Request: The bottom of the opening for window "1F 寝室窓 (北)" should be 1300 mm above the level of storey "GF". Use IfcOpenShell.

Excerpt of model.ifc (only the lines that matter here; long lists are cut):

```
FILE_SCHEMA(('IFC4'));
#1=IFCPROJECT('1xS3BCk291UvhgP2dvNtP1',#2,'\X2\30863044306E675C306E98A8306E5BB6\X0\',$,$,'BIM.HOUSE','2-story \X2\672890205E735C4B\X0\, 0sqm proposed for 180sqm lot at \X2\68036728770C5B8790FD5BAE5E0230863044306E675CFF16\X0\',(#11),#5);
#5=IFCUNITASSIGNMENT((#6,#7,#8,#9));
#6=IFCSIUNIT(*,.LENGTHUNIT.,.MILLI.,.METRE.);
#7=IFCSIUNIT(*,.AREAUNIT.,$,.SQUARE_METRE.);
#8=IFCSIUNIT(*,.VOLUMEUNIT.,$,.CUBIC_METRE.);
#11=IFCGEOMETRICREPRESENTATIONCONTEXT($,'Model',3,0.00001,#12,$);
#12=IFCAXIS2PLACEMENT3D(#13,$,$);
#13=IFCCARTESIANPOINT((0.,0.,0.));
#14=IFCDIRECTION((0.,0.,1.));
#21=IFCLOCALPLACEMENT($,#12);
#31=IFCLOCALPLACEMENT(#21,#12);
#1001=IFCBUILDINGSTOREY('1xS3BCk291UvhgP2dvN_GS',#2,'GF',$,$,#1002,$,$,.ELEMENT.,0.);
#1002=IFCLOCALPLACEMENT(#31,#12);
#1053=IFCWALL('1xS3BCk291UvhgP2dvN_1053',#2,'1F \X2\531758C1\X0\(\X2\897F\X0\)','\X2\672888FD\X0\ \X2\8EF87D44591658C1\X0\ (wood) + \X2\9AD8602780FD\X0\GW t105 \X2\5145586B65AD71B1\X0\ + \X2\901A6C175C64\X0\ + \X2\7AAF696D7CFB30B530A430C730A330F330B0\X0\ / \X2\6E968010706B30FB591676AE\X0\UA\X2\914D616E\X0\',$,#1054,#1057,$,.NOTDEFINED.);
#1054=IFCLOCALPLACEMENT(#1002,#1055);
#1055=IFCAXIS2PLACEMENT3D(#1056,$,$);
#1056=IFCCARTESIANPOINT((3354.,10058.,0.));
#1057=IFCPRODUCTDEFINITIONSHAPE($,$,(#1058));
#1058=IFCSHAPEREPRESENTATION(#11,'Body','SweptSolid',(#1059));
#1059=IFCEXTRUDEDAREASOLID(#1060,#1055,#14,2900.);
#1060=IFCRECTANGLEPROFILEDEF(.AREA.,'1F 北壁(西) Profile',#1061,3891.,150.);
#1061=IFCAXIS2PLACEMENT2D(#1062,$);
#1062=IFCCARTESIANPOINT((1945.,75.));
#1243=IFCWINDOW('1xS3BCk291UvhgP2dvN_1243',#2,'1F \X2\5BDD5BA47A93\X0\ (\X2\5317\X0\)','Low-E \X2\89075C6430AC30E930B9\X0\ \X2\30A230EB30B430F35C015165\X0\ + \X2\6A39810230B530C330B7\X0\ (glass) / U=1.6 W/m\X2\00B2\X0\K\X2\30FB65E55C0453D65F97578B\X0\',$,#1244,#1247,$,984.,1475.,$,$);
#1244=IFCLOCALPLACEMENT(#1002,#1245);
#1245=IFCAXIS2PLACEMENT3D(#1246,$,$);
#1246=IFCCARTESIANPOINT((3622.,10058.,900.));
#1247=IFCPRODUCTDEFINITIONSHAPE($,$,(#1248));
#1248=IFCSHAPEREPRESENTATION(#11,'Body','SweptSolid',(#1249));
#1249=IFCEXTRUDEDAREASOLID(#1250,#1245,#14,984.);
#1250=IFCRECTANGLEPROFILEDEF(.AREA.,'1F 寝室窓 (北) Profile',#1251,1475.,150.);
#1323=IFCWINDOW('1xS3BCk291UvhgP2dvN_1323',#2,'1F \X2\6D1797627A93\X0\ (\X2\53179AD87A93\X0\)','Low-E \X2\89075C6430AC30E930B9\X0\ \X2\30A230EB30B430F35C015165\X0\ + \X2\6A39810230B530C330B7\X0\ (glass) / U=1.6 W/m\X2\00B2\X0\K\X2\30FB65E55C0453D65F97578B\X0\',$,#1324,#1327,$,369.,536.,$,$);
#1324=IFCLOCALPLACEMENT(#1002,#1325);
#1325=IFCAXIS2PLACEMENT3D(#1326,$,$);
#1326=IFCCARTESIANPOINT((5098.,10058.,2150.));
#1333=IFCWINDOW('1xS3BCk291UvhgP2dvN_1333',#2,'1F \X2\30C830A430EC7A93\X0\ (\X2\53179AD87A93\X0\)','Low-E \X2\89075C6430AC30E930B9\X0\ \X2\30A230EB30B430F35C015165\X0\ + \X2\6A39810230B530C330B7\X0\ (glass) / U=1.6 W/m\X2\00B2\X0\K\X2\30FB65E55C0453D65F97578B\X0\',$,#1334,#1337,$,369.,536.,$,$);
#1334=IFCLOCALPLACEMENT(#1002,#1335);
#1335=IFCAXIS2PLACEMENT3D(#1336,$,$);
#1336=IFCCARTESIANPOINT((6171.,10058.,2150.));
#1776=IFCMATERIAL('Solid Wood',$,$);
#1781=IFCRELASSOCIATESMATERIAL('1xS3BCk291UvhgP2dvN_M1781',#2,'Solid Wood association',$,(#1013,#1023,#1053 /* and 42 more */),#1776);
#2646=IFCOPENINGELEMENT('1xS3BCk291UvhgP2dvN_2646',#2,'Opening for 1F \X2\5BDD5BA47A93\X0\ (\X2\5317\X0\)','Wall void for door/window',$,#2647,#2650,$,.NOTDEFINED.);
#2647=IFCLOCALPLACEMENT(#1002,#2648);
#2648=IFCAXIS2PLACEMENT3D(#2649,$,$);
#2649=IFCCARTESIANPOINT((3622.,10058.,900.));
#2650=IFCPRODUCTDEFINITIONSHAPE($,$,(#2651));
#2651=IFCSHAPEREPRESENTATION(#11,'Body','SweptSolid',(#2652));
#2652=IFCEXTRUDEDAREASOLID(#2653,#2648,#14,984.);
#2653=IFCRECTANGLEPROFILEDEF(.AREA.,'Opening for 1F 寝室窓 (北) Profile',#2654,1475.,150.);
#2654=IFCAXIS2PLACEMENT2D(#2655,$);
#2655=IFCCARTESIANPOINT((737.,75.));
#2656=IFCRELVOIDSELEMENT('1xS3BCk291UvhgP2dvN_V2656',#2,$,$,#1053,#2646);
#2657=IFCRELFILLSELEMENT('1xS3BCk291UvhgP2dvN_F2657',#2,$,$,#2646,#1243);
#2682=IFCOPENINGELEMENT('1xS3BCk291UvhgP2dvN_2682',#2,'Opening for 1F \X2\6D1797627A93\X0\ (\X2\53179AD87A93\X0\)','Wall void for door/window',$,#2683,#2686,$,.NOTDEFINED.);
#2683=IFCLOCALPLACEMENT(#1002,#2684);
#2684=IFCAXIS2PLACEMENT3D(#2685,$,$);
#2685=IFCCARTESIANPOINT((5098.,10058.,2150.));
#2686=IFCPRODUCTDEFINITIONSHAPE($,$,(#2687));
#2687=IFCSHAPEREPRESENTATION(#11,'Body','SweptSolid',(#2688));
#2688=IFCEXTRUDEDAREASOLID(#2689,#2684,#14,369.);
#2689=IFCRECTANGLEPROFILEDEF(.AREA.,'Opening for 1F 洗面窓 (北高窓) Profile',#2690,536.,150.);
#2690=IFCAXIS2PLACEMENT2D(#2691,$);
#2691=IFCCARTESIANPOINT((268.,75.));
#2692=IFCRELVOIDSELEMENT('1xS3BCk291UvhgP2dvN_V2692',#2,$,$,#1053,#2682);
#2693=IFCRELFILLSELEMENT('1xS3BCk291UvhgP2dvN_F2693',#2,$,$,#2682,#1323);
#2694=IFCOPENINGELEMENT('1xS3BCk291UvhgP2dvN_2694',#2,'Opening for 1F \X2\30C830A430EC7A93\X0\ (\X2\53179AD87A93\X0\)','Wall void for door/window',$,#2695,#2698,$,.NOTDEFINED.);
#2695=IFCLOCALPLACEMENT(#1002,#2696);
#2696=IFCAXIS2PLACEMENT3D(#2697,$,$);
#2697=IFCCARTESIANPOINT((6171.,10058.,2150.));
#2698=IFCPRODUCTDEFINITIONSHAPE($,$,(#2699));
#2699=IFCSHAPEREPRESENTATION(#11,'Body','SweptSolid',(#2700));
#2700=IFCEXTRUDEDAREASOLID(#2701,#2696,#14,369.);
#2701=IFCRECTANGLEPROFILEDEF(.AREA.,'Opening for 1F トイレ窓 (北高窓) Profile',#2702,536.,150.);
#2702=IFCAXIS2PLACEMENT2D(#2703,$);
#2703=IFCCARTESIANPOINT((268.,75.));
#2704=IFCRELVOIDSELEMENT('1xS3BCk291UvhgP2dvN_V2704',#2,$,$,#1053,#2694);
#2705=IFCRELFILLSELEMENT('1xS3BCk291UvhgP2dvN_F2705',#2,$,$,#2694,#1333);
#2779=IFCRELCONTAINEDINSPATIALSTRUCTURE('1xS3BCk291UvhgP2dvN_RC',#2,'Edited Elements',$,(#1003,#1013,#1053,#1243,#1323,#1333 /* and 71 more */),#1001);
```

```python
import numpy as np
import ifcopenshell
import ifcopenshell.api.geometry
import ifcopenshell.geom
import ifcopenshell.util.element
import ifcopenshell.util.placement
import ifcopenshell.util.shape
import ifcopenshell.util.unit

model = ifcopenshell.open("model.ifc")
unit_scale = ifcopenshell.util.unit.calculate_unit_scale(model)

window = model.by_guid("1xS3BCk291UvhgP2dvN_1243")
opening = window.FillsVoids[0].RelatingOpeningElement
storey = ifcopenshell.util.element.get_container(window, ifc_class="IfcBuildingStorey")
level = ifcopenshell.util.placement.get_local_placement(storey.ObjectPlacement)[2, 3]

# The opening's origin need not be at the sill, so measure its lowest point.
shape = ifcopenshell.geom.create_shape(ifcopenshell.geom.settings(), opening)
bottom = ifcopenshell.util.shape.get_shape_bottom_elevation(shape, shape.geometry) / unit_scale
dz = level + 1.3 / unit_scale - bottom

shift = np.array([0.0, 0.0, dz])
# The window is not placed relative to its opening, so move both.
for product in (opening, window):
    matrix = ifcopenshell.util.placement.get_local_placement(product.ObjectPlacement)
    matrix[:3, 3] += shift
    ifcopenshell.api.geometry.edit_object_placement(model, product=product, matrix=matrix, is_si=False)

print(f"moved by {dz * unit_scale:+.3f} m")

model.write("model_edited.ifc")
```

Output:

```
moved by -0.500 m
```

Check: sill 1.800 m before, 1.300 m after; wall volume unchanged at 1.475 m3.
